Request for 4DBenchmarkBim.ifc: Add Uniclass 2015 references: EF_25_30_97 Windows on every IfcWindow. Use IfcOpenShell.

First a look at what the model holds.

```python
import ifcopenshell

model = ifcopenshell.open("4DBenchmarkBim.ifc")
print(model.schema)
print("classifications:", [c.Name for c in model.by_type("IfcClassification")])
for ifc_class in ("IfcDoor", "IfcRoof", "IfcStair", "IfcWall", "IfcWindow"):
    print(ifc_class, len(model.by_type(ifc_class)))
```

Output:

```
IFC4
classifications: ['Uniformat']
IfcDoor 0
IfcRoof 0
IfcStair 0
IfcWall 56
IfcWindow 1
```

```python
import ifcopenshell
import ifcopenshell.api.classification

model = ifcopenshell.open("4DBenchmarkBim.ifc")

system = ifcopenshell.api.classification.add_classification(model, classification="Uniclass 2015")

codes = {
    "IfcWindow": ("EF_25_30_97", "Windows"),
}
for ifc_class, (code, name) in codes.items():
    products = model.by_type(ifc_class)
    ifcopenshell.api.classification.add_reference(
        model, products=products, classification=system, identification=code, name=name
    )
    print(code, len(products))

model.write("4DBenchmarkBim_edited.ifc")
```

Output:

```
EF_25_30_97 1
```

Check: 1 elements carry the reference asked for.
